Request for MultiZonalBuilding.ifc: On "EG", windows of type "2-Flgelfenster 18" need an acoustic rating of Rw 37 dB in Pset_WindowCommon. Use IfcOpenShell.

First a look at what the model holds.

```python
import ifcopenshell
import ifcopenshell.util.element

model = ifcopenshell.open("MultiZonalBuilding.ifc")
print(model.schema)
storey = next(s for s in model.by_type("IfcBuildingStorey") if s.Name == "EG")
windows = [e for e in ifcopenshell.util.element.get_decomposition(storey) if e.is_a("IfcWindow")]
seen = {}
for e in windows:
    element_type = ifcopenshell.util.element.get_type(e)
    key = (element_type.Name if element_type != e and element_type else None, ifcopenshell.util.element.get_pset(e, "Pset_WindowCommon", "AcousticRating"))
    seen[key] = seen.get(key, 0) + 1
for (name, value), count in sorted(seen.items(), key=str):
    print(count, "x", name, "|", value)
```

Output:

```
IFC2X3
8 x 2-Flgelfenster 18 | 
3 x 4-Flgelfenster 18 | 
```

```python
import ifcopenshell
import ifcopenshell.api.pset
import ifcopenshell.util.element

model = ifcopenshell.open("MultiZonalBuilding.ifc")

storey = next(s for s in model.by_type("IfcBuildingStorey") if s.Name == "EG")
windows = [e for e in ifcopenshell.util.element.get_decomposition(storey) if e.is_a("IfcWindow")]

count = 0
for e in windows:
    element_type = ifcopenshell.util.element.get_type(e)
    if element_type in (None, e) or element_type.Name != '2-Fl\x9fgelfenster 18':
        continue
    # add_pset returns the element's existing set when there is one.
    pset = ifcopenshell.api.pset.add_pset(model, product=e, name="Pset_WindowCommon")
    ifcopenshell.api.pset.edit_pset(model, pset=pset, properties={"AcousticRating": "Rw 37 dB"})
    count += 1

print(count, "windows updated")

model.write("MultiZonalBuilding_v2.ifc")
```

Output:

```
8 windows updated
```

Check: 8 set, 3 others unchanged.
